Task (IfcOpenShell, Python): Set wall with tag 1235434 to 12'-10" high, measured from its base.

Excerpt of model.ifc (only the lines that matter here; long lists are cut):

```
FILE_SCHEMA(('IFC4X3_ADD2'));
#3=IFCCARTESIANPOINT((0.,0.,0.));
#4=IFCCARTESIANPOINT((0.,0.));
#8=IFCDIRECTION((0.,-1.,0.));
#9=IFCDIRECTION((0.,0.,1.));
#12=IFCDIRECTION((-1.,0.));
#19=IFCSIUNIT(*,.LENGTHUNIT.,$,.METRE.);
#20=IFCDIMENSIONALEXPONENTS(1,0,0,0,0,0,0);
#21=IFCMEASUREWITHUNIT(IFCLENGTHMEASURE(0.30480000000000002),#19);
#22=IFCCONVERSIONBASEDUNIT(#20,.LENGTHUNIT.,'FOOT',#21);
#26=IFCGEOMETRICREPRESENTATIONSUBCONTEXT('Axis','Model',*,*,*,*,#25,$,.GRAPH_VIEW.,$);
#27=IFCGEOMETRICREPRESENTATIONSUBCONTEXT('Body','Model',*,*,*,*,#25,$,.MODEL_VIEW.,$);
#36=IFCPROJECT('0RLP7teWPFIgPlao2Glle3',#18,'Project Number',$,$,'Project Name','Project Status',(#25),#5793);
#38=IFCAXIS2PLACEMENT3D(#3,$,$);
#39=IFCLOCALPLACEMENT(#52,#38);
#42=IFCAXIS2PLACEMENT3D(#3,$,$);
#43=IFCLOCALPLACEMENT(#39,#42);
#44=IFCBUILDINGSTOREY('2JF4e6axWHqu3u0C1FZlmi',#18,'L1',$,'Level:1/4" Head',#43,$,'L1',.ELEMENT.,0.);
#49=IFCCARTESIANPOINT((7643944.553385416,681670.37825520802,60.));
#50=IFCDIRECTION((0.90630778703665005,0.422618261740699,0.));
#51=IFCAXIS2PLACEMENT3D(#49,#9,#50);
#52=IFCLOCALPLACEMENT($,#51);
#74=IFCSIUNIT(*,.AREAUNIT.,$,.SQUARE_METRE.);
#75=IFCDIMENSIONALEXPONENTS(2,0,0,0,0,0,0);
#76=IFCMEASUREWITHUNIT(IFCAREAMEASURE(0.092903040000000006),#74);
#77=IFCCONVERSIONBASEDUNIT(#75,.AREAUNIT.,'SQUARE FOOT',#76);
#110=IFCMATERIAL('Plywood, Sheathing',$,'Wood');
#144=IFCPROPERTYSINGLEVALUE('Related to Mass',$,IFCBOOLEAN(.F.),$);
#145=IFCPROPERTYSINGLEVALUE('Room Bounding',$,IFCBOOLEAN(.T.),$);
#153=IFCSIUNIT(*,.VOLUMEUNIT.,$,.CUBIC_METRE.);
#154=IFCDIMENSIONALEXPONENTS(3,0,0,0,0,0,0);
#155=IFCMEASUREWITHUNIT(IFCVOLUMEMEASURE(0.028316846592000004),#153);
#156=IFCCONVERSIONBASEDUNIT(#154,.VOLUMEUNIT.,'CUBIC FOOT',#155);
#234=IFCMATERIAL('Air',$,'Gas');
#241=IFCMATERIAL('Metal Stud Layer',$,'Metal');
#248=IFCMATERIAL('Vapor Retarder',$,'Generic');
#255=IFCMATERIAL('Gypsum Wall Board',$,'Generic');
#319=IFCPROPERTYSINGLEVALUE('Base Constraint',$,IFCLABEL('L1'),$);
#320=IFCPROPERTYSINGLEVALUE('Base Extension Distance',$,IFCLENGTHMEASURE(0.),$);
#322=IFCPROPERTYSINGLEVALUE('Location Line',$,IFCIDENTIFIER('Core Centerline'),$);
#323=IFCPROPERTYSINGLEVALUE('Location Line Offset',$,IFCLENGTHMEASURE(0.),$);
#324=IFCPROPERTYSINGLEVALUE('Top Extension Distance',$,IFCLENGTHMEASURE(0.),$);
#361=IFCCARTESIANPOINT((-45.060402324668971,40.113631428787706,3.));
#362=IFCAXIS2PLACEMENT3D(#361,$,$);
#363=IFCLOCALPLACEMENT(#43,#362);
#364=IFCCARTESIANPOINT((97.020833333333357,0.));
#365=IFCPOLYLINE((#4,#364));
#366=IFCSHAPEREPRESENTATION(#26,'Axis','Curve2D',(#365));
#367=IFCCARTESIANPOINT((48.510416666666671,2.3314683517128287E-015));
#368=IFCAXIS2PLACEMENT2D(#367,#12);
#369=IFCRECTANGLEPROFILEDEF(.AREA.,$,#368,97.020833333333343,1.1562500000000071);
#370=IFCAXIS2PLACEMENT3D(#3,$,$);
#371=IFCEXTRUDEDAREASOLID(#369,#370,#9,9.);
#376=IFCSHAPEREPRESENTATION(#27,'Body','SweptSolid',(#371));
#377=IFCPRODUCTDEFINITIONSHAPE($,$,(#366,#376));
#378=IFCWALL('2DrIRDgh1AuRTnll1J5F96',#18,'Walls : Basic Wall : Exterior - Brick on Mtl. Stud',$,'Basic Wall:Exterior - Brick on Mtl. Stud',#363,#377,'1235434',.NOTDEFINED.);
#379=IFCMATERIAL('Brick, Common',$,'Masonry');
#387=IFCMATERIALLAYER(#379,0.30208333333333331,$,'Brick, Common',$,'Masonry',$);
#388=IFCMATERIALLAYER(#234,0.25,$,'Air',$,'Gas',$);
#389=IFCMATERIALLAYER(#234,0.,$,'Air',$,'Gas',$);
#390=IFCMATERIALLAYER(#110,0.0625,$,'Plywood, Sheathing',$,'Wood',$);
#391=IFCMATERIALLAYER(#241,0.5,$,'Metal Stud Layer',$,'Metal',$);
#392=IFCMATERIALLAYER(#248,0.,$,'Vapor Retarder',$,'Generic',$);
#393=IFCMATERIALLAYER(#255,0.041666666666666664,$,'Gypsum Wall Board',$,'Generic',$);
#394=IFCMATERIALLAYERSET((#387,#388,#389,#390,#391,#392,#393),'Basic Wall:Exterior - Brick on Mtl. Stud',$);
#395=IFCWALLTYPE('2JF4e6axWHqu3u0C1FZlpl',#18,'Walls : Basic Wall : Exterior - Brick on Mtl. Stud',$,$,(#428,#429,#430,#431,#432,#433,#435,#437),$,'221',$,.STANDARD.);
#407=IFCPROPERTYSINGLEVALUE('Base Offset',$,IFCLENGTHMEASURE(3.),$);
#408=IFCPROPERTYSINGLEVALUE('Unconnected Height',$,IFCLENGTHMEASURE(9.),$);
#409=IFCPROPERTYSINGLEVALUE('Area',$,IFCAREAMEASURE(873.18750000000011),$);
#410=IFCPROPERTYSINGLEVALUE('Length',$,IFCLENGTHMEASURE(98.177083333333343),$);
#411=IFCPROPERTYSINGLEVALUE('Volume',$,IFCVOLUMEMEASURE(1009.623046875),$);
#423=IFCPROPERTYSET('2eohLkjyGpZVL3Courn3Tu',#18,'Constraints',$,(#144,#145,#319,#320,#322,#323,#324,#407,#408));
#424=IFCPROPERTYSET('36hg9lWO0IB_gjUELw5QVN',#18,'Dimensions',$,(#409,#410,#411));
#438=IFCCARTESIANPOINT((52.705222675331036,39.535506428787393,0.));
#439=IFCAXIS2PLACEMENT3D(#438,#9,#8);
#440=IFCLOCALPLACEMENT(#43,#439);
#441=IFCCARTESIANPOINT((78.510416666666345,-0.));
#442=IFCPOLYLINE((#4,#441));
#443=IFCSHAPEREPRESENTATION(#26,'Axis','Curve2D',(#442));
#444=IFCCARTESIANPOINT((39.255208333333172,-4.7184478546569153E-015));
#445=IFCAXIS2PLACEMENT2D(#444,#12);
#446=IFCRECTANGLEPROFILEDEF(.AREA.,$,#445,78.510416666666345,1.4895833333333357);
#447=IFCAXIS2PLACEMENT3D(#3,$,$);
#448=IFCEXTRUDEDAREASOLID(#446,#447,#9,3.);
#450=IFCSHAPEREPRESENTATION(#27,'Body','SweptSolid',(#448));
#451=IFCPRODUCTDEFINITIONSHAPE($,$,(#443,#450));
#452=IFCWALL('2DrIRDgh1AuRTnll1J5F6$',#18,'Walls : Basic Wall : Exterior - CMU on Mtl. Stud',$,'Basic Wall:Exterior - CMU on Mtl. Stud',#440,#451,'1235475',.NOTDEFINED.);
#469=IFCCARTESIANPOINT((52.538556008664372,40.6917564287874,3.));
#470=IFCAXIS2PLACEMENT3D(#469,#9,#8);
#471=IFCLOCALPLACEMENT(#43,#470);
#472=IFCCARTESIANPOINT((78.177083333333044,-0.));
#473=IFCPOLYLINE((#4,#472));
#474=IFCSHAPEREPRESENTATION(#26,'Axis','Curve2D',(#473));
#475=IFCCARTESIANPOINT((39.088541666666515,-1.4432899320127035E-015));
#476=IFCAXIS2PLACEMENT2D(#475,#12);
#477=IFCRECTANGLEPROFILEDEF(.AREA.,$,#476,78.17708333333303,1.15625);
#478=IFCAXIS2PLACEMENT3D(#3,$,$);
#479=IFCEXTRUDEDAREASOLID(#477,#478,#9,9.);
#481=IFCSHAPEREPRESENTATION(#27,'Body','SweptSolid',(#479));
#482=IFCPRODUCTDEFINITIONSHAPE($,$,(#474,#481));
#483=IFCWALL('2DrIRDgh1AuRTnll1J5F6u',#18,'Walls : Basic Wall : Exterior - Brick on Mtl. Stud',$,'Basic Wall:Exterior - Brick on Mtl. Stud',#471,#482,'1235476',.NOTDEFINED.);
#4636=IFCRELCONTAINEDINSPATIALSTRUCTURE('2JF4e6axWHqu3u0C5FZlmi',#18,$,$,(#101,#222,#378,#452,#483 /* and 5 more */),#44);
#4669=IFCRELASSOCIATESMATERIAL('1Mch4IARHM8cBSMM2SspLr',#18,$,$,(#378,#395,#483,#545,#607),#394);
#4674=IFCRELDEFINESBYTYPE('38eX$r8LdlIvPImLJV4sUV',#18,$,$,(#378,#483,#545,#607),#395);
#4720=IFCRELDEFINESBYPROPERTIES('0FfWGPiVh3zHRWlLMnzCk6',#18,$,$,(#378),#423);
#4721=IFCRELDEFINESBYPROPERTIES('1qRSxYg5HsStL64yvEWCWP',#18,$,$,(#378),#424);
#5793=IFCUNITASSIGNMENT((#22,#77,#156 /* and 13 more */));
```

```python
import ifcopenshell
import ifcopenshell.api.pset
import ifcopenshell.geom
import ifcopenshell.util.element
import ifcopenshell.util.representation
import ifcopenshell.util.shape
import ifcopenshell.util.unit

model = ifcopenshell.open("model.ifc")
unit_scale = ifcopenshell.util.unit.calculate_unit_scale(model)
area_scale = ifcopenshell.util.unit.calculate_unit_scale(model, "AREAUNIT")
volume_scale = ifcopenshell.util.unit.calculate_unit_scale(model, "VOLUMEUNIT")
settings = ifcopenshell.geom.settings()


def volume(element):
    """Net volume in cubic metres, openings subtracted."""
    shape = ifcopenshell.geom.create_shape(settings, element)
    return ifcopenshell.util.shape.get_volume(shape.geometry)


wall = model.by_id(378)
before = volume(wall)

body = ifcopenshell.util.representation.get_representation(wall, "Model", "Body")
solid = body.Items[0]
old_height = solid.Depth
solid.Depth = 154 * 0.0254 / unit_scale
after = volume(wall)
thickness = 0.3524  # wall thickness in metres

# Update the stored height, areas and volumes.
pset = model.by_id(ifcopenshell.util.element.get_pset(wall, "Constraints", should_inherit=False)["id"])
ifcopenshell.api.pset.edit_pset(model, pset=pset, properties={
    "Unconnected Height": model.create_entity("IfcLengthMeasure", solid.Depth),
})
pset = model.by_id(ifcopenshell.util.element.get_pset(wall, "Dimensions", should_inherit=False)["id"])
ifcopenshell.api.pset.edit_pset(model, pset=pset, properties={
    "Area": model.create_entity("IfcAreaMeasure", after / thickness / area_scale),
    "Volume": model.create_entity("IfcVolumeMeasure", after / volume_scale),
})

print(f"height {old_height:g} -> {solid.Depth:g}, volume {before:.3f} -> {after:.3f} m3")

model.write("model-out.ifc")
```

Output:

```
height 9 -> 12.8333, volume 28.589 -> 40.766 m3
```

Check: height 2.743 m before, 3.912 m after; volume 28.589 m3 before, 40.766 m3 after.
